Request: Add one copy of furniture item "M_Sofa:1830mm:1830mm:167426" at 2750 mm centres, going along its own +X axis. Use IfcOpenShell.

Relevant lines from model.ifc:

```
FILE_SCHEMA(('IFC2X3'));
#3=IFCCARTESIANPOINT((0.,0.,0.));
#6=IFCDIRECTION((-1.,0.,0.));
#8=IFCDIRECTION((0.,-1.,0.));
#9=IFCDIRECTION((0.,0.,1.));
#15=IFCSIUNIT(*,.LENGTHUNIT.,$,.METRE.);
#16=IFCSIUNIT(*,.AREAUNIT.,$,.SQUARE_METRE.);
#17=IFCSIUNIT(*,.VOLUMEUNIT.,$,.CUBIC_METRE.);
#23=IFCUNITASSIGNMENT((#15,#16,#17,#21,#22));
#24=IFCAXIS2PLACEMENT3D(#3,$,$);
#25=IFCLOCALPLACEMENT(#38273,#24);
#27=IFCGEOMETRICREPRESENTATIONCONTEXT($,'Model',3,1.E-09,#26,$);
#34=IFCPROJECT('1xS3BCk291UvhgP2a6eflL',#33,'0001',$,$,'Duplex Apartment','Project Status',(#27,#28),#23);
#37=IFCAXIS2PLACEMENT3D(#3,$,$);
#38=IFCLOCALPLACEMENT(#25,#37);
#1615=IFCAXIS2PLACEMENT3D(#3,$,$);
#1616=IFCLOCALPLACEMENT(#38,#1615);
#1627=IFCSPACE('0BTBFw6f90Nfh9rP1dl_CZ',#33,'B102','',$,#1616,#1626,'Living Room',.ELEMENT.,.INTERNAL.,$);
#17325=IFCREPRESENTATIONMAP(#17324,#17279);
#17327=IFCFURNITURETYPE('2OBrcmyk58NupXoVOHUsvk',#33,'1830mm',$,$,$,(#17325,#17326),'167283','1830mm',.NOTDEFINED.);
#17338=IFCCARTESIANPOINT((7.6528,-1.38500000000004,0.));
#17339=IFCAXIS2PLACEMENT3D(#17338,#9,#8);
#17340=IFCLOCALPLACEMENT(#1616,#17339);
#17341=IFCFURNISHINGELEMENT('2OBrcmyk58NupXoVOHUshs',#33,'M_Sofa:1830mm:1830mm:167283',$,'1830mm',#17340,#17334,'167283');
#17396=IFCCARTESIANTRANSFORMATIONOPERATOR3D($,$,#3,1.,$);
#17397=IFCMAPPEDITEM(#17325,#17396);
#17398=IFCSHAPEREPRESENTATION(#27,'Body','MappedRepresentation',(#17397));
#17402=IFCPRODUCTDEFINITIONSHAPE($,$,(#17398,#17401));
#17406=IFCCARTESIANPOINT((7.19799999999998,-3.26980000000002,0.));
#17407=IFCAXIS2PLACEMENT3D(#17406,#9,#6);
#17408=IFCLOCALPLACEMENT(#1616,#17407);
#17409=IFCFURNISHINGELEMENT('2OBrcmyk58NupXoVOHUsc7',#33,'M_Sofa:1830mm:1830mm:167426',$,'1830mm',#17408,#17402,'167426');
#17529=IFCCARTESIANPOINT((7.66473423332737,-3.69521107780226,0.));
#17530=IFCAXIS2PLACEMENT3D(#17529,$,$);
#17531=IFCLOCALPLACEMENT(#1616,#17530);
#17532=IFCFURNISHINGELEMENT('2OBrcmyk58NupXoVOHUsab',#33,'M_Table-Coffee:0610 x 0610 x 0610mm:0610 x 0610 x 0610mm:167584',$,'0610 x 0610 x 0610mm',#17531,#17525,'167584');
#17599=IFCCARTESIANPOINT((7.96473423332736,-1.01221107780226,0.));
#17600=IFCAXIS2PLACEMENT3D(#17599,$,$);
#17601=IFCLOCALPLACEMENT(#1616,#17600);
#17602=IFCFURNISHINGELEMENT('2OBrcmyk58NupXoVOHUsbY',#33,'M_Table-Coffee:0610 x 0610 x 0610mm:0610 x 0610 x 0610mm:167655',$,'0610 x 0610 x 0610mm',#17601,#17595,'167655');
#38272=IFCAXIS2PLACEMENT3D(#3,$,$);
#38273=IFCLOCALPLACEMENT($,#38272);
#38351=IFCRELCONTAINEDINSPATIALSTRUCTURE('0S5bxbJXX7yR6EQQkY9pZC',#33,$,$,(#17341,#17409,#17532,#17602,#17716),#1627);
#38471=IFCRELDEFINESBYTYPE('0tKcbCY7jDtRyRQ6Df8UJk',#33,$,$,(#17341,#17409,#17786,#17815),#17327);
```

```python
import ifcopenshell
import ifcopenshell.api.geometry
import ifcopenshell.api.root
import ifcopenshell.util.element
import ifcopenshell.util.placement
import ifcopenshell.util.unit

model = ifcopenshell.open("model.ifc")
unit_scale = ifcopenshell.util.unit.calculate_unit_scale(model)


def reuse_history(source, copy):
    """copy_class also copies each property set's owner history, people and application; keep the originals."""
    for rel in copy.IsDefinedBy:
        if rel.is_a("IfcRelDefinesByProperties") and (history := rel.RelatingPropertyDefinition.OwnerHistory):
            rel.RelatingPropertyDefinition.OwnerHistory = source.OwnerHistory
            ifcopenshell.util.element.remove_deep2(model, history)


source = model.by_guid("2OBrcmyk58NupXoVOHUsc7")
base = ifcopenshell.util.placement.get_local_placement(source.ObjectPlacement)
step = base[:3, 0] * 2.75 / unit_scale

for i in range(1, 2):
    copy = ifcopenshell.api.root.copy_class(model, product=source)
    copy.Representation = ifcopenshell.util.element.copy_deep(
        model, source.Representation, exclude=["IfcGeometricRepresentationContext", "IfcRepresentationMap"]
    )
    copy.Name = "M_Sofa:1830mm:1830mm"
    copy.Tag = None
    reuse_history(source, copy)
    matrix = base.copy()
    matrix[:3, 3] += i * step
    print("added at", matrix[:3, 3].round(3) + 0.0)
    ifcopenshell.api.geometry.edit_object_placement(model, product=copy, matrix=matrix, is_si=False)

model.write("model_v2.ifc")
```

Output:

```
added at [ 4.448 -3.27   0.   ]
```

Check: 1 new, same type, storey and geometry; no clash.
